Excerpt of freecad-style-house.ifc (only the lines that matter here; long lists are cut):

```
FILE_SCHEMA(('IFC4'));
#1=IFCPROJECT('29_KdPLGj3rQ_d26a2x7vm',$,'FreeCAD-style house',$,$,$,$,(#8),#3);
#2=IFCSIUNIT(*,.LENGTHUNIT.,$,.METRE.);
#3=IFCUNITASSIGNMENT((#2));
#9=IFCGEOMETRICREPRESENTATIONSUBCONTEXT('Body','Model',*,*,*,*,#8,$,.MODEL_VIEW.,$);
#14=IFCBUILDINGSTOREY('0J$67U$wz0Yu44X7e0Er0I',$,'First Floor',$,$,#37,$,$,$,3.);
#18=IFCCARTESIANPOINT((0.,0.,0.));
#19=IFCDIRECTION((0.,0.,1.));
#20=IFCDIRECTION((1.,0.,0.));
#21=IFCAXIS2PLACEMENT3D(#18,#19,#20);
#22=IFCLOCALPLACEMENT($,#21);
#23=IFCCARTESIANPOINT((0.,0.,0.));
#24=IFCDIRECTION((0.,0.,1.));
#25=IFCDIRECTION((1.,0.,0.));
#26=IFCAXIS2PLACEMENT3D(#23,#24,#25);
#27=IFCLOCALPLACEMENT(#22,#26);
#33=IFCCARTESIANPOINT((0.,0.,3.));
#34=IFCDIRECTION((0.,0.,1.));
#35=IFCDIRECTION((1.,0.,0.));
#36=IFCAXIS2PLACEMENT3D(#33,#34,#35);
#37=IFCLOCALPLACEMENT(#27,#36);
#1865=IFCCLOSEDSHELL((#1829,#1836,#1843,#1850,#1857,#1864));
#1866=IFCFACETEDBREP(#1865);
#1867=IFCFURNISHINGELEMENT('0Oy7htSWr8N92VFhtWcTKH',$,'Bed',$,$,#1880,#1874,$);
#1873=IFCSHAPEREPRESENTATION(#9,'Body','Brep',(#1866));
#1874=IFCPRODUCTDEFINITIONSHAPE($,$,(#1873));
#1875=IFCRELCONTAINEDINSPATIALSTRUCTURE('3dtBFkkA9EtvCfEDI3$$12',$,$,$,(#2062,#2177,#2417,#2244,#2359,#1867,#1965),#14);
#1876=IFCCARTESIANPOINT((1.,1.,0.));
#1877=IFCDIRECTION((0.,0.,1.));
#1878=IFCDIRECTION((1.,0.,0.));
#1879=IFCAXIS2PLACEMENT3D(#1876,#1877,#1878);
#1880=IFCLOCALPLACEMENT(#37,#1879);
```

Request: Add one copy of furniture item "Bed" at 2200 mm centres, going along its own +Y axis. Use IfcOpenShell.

```python
import ifcopenshell
import ifcopenshell.api.geometry
import ifcopenshell.api.root
import ifcopenshell.util.element
import ifcopenshell.util.placement
import ifcopenshell.util.unit

model = ifcopenshell.open("freecad-style-house.ifc")
unit_scale = ifcopenshell.util.unit.calculate_unit_scale(model)

source = model.by_id(1867)
base = ifcopenshell.util.placement.get_local_placement(source.ObjectPlacement)
step = base[:3, 1] * 2.2 / unit_scale

for i in range(1, 2):
    copy = ifcopenshell.api.root.copy_class(model, product=source)
    copy.Representation = ifcopenshell.util.element.copy_deep(
        model, source.Representation, exclude=["IfcGeometricRepresentationContext", "IfcRepresentationMap"]
    )
    matrix = base.copy()
    matrix[:3, 3] += i * step
    print("added at", matrix[:3, 3].round(3) + 0.0)
    ifcopenshell.api.geometry.edit_object_placement(model, product=copy, matrix=matrix, is_si=False)

model.write("freecad-style-house_edited.ifc")
```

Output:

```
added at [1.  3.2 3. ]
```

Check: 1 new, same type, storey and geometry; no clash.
